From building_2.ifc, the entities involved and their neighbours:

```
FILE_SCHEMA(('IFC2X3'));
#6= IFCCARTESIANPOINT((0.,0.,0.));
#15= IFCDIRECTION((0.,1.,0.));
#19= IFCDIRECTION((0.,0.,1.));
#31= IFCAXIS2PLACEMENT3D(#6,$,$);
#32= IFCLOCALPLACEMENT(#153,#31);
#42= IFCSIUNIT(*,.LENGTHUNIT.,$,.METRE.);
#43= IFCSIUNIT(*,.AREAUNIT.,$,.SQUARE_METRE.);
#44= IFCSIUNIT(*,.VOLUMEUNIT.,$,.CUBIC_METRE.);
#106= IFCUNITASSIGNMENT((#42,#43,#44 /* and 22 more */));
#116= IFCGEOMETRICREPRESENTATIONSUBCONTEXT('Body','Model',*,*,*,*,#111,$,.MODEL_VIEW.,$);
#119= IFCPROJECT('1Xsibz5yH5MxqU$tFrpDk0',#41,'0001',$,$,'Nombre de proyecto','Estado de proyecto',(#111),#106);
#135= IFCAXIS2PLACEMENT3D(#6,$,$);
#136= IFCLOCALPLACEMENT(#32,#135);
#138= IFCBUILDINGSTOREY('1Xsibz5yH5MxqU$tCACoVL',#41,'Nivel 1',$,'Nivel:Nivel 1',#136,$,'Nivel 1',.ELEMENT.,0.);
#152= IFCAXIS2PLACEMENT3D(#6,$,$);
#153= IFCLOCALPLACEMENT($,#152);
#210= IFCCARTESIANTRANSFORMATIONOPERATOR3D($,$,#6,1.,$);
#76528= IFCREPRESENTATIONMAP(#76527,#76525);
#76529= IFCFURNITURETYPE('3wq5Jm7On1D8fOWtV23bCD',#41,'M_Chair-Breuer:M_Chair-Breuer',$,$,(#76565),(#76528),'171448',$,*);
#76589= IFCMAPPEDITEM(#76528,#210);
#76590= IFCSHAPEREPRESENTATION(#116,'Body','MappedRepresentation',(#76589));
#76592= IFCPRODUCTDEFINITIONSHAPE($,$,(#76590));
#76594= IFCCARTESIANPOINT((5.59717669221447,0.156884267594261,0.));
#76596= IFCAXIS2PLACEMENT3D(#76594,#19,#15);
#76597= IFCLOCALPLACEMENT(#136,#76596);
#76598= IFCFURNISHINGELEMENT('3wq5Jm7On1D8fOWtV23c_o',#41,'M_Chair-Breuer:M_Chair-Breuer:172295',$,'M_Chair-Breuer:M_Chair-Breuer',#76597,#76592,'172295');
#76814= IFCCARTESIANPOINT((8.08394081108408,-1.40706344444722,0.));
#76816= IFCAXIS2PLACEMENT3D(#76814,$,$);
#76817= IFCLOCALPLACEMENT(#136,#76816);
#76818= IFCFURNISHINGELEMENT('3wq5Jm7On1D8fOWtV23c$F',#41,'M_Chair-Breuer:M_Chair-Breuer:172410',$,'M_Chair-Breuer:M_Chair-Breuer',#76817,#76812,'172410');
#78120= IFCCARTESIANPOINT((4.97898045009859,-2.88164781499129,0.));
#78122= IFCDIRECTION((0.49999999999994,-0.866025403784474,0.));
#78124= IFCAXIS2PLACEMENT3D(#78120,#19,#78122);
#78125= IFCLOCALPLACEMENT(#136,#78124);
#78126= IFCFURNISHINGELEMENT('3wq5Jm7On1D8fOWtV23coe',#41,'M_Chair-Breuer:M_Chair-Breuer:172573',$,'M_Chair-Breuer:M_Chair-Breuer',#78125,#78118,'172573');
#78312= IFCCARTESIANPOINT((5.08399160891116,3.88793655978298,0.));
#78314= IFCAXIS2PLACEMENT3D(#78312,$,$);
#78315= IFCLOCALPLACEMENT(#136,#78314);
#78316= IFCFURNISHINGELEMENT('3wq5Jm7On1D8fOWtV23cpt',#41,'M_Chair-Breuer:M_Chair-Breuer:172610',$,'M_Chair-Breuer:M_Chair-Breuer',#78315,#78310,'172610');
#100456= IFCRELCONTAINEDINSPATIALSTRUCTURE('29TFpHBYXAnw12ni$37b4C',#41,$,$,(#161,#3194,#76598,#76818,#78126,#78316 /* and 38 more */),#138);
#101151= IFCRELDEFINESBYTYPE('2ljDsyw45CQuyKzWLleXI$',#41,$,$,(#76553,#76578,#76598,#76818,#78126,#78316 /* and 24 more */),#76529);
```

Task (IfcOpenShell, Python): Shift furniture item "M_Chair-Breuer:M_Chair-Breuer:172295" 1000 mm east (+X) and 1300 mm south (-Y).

```python
import ifcopenshell
import ifcopenshell.api.geometry
import ifcopenshell.util.placement

model = ifcopenshell.open("building_2.ifc")

item = model.by_id(76598)
matrix = ifcopenshell.util.placement.get_local_placement(item.ObjectPlacement)
matrix[0, 3] += 1.0
matrix[1, 3] -= 1.3
ifcopenshell.api.geometry.edit_object_placement(model, product=item, matrix=matrix, is_si=False)

print(ifcopenshell.util.placement.get_local_placement(item.ObjectPlacement).round(3) + 0.0)

model.write("building_2-out.ifc")
```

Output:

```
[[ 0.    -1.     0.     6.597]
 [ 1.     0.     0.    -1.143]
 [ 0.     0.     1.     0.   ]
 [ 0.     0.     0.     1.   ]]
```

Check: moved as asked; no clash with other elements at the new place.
